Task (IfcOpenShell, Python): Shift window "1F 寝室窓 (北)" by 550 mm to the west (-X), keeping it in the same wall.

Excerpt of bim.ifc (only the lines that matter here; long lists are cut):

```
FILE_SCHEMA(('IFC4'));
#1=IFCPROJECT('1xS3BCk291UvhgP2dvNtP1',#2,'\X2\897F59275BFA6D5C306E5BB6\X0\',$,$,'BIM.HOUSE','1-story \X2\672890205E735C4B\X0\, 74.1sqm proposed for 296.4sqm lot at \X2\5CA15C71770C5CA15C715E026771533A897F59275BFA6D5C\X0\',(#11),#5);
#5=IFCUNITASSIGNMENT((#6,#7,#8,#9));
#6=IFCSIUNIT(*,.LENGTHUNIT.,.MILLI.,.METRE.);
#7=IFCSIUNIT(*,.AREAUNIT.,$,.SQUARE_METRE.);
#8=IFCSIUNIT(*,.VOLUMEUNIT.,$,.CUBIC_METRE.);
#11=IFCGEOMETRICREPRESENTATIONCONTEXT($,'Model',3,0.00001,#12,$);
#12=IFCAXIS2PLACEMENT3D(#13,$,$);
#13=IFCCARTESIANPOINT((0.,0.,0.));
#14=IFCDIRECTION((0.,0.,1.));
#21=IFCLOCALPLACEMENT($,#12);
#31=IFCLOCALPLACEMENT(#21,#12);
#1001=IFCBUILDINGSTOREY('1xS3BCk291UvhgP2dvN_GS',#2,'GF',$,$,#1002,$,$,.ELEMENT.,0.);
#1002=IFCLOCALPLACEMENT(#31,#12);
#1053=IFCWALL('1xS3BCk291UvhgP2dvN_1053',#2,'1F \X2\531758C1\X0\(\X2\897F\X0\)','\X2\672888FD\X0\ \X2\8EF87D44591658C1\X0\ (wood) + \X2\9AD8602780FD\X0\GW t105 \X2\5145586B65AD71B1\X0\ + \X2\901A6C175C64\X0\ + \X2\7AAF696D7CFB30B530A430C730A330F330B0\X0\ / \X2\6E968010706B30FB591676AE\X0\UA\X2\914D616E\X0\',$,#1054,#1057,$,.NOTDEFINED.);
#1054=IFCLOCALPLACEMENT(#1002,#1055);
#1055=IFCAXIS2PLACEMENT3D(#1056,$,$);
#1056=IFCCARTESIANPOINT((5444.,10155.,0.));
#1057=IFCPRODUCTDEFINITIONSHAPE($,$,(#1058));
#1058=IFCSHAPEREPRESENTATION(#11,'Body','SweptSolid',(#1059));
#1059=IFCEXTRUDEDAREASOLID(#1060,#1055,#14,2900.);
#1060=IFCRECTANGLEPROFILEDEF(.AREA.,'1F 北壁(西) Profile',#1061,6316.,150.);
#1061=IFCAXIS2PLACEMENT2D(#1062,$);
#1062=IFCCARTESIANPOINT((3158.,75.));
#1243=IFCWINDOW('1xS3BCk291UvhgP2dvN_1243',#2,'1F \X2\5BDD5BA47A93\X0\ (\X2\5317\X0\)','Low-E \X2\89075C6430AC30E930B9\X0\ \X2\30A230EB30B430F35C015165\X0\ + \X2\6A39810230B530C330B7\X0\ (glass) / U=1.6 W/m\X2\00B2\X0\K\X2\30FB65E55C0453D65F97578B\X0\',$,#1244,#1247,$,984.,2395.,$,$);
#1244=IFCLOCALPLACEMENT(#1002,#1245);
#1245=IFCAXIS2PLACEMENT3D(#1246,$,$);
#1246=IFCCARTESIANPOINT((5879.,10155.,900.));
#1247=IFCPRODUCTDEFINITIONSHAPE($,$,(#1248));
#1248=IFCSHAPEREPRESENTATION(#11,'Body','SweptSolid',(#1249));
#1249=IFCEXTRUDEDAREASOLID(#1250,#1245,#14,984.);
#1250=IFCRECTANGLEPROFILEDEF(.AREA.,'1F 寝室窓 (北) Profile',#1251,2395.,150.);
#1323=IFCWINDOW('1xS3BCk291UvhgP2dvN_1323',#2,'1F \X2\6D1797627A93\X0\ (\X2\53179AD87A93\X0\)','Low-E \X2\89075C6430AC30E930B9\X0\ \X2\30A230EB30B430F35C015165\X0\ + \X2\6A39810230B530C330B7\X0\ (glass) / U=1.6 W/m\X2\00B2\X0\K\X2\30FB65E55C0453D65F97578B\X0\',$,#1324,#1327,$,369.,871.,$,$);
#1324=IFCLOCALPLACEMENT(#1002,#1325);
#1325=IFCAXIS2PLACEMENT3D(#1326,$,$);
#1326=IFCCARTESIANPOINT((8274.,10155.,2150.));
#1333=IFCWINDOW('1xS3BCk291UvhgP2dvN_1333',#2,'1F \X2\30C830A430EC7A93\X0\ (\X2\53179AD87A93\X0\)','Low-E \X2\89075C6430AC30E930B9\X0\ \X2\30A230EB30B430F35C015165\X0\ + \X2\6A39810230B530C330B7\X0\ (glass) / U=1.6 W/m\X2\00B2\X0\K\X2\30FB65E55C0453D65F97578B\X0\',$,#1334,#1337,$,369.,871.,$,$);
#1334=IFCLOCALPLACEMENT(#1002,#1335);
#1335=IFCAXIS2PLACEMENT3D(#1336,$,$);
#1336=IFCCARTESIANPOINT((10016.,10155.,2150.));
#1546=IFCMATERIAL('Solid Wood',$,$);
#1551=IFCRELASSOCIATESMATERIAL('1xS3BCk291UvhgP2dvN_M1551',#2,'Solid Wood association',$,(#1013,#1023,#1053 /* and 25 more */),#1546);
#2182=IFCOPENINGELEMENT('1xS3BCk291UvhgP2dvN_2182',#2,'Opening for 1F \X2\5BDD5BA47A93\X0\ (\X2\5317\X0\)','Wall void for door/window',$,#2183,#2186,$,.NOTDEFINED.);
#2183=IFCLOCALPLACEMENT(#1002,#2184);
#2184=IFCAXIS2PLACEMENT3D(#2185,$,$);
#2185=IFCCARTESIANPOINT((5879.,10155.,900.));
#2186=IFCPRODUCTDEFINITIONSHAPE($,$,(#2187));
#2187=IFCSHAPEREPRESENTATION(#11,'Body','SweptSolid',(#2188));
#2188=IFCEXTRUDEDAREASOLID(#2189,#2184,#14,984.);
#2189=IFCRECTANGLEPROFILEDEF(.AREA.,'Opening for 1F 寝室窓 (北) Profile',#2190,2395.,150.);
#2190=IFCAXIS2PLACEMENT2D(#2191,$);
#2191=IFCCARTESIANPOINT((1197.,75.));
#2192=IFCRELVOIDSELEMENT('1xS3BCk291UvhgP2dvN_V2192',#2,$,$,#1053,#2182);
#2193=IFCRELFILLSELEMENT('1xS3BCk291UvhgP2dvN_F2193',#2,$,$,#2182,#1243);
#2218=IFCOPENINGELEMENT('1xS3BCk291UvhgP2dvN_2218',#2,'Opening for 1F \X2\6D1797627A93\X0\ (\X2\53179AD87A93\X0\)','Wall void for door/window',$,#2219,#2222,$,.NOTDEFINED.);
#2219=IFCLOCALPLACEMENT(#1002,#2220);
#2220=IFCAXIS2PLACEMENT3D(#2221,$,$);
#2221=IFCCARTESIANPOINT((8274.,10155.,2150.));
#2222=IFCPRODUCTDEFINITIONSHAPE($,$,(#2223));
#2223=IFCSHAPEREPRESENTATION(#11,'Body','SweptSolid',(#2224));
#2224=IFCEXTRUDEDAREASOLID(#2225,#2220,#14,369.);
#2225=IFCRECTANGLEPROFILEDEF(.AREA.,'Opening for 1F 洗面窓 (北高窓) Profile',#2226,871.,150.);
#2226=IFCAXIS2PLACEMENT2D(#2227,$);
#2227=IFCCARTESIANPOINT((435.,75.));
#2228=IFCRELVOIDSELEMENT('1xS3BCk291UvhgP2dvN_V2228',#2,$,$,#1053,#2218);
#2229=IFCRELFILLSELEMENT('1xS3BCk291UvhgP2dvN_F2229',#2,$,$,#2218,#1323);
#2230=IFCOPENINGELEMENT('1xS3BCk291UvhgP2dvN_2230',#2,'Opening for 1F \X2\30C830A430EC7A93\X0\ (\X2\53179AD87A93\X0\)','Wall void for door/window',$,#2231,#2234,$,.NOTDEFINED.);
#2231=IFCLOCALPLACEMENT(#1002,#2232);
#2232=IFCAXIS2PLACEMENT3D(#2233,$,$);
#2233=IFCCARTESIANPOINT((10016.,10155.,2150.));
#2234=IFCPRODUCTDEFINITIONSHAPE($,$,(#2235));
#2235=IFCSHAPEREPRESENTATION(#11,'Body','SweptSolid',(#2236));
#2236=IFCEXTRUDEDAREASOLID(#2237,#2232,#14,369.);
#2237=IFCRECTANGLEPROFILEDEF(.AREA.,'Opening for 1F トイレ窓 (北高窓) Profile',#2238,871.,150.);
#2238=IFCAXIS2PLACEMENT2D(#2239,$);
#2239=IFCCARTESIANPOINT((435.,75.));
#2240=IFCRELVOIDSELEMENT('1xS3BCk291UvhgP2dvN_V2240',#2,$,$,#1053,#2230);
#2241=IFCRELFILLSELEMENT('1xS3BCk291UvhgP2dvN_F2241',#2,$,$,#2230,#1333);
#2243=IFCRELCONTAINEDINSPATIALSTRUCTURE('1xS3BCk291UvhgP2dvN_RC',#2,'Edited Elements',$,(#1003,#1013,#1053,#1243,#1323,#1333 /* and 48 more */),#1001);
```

```python
import ifcopenshell
import ifcopenshell.api.geometry
import ifcopenshell.util.placement
import ifcopenshell.util.unit

model = ifcopenshell.open("bim.ifc")
unit_scale = ifcopenshell.util.unit.calculate_unit_scale(model)

window = model.by_id(1243)
opening = window.FillsVoids[0].RelatingOpeningElement
wall = opening.VoidsElements[0].RelatingBuildingElement

wall_matrix = ifcopenshell.util.placement.get_local_placement(wall.ObjectPlacement)
shift = wall_matrix[:3, 0] * -0.55 / unit_scale
before = ifcopenshell.util.placement.get_local_placement(window.ObjectPlacement)[:3, 3].copy()

# The window is not placed relative to its opening, so move both.
for product in (opening, window):
    matrix = ifcopenshell.util.placement.get_local_placement(product.ObjectPlacement)
    matrix[:3, 3] += shift
    ifcopenshell.api.geometry.edit_object_placement(model, product=product, matrix=matrix, is_si=False)

after = ifcopenshell.util.placement.get_local_placement(window.ObjectPlacement)[:3, 3]
print("window moved by", (after - before).round(3) + 0.0)

model.write("bim-out.ifc")
```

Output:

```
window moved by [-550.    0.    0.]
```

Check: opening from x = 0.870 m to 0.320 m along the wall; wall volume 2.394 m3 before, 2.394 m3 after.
